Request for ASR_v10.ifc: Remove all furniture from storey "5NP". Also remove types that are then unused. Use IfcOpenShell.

First a look at what the model holds.

```python
import ifcopenshell
import ifcopenshell.util.element

model = ifcopenshell.open("ASR_v10.ifc")
print(model.schema)
storey = next(s for s in model.by_type("IfcBuildingStorey") if s.Name == "5NP")
furniture = [e for e in ifcopenshell.util.element.get_decomposition(storey) if e.is_a("IfcFurnishingElement")]
seen = {}
for e in furniture:
    element_type = ifcopenshell.util.element.get_type(e)
    name = element_type.Name if element_type not in (None, e) else None
    seen[name] = seen.get(name, 0) + 1
for name, count in sorted(seen.items(), key=str):
    print(count, "x", name)
```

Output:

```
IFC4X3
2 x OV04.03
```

```python
import ifcopenshell
import ifcopenshell.api.root
import ifcopenshell.util.element

model = ifcopenshell.open("ASR_v10.ifc")

storey = next(s for s in model.by_type("IfcBuildingStorey") if s.Name == "5NP")
furniture = [e for e in ifcopenshell.util.element.get_decomposition(storey) if e.is_a("IfcFurnishingElement")]
types = {ifcopenshell.util.element.get_type(e) for e in furniture} - {None, *furniture}

for e in furniture:
    ifcopenshell.api.root.remove_product(model, product=e)
print(len(furniture), "removed")

unused = [t for t in types if not ifcopenshell.util.element.get_types(t)]
for t in unused:
    ifcopenshell.api.root.remove_product(model, product=t)
print(len(unused), "unused types removed")

model.write("ASR_v10-out.ifc")
```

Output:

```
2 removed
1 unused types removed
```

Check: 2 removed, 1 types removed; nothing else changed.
